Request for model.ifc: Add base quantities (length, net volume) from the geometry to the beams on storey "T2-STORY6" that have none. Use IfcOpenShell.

First a look at what the model holds.

```python
import ifcopenshell
import ifcopenshell.util.element
import ifcopenshell.util.unit

model = ifcopenshell.open("model.ifc")
print(model.schema)
for unit_type in ("LENGTHUNIT", "AREAUNIT", "VOLUMEUNIT"):
    print(unit_type, ifcopenshell.util.unit.calculate_unit_scale(model, unit_type))
storey = next(s for s in model.by_type("IfcBuildingStorey") if s.Name == "T2-STORY6")
beams = [e for e in ifcopenshell.util.element.get_decomposition(storey) if e.is_a("IfcBeam")]
for e in sorted(beams, key=lambda e: e.id()):
    print(e.id(), e.is_a(), e.Name, list(ifcopenshell.util.element.get_psets(e, qtos_only=True)), sep=" | ")
```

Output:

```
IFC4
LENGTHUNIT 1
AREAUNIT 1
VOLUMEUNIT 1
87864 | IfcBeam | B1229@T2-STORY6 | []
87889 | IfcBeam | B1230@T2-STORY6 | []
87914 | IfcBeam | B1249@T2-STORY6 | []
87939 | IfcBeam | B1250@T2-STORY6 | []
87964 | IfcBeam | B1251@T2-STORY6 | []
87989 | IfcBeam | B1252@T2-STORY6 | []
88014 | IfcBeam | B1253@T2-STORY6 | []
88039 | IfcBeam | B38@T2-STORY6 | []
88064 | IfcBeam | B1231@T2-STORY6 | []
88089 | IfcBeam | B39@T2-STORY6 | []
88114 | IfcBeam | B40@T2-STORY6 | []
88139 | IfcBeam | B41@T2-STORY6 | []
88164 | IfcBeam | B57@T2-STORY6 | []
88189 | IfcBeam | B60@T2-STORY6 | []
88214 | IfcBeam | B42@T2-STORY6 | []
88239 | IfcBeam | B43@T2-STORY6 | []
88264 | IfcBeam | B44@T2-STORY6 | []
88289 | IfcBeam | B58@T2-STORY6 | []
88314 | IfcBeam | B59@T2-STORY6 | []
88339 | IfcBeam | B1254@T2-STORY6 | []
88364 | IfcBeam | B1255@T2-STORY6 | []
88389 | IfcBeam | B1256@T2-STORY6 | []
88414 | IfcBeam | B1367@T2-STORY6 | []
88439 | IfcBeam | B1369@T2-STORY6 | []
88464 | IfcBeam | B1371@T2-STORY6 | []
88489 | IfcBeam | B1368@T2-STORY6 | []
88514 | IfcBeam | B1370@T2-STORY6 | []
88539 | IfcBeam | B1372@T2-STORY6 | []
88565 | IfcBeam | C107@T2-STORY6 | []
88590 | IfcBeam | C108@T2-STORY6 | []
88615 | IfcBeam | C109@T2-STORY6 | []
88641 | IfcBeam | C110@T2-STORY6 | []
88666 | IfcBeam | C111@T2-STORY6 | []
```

```python
import ifcopenshell
import ifcopenshell.api.pset
import ifcopenshell.geom
import ifcopenshell.util.element
import ifcopenshell.util.shape
import ifcopenshell.util.unit

model = ifcopenshell.open("model.ifc")
unit_scale = ifcopenshell.util.unit.calculate_unit_scale(model)
volume_scale = ifcopenshell.util.unit.calculate_unit_scale(model, "VOLUMEUNIT")
settings = ifcopenshell.geom.settings()

storey = next(s for s in model.by_type("IfcBuildingStorey") if s.Name == "T2-STORY6")
beams = [e for e in ifcopenshell.util.element.get_decomposition(storey) if e.is_a("IfcBeam")]

for e in sorted(beams, key=lambda e: e.id()):
    if ifcopenshell.util.element.get_psets(e, qtos_only=True, should_inherit=False):
        continue
    # Geometry comes back in metres, in the element's own axes.
    shape = ifcopenshell.geom.create_shape(settings, e)
    values = {
        "Length": ifcopenshell.util.shape.get_max_xyz(shape.geometry) / unit_scale,
        "NetVolume": ifcopenshell.util.shape.get_volume(shape.geometry) / volume_scale,
    }
    qto = ifcopenshell.api.pset.add_qto(model, product=e, name="Qto_BeamBaseQuantities")
    ifcopenshell.api.pset.edit_qto(model, qto=qto, properties=values)
    print(e.id(), {k: round(v, 3) for k, v in values.items()})

model.write("model_updated.ifc")
```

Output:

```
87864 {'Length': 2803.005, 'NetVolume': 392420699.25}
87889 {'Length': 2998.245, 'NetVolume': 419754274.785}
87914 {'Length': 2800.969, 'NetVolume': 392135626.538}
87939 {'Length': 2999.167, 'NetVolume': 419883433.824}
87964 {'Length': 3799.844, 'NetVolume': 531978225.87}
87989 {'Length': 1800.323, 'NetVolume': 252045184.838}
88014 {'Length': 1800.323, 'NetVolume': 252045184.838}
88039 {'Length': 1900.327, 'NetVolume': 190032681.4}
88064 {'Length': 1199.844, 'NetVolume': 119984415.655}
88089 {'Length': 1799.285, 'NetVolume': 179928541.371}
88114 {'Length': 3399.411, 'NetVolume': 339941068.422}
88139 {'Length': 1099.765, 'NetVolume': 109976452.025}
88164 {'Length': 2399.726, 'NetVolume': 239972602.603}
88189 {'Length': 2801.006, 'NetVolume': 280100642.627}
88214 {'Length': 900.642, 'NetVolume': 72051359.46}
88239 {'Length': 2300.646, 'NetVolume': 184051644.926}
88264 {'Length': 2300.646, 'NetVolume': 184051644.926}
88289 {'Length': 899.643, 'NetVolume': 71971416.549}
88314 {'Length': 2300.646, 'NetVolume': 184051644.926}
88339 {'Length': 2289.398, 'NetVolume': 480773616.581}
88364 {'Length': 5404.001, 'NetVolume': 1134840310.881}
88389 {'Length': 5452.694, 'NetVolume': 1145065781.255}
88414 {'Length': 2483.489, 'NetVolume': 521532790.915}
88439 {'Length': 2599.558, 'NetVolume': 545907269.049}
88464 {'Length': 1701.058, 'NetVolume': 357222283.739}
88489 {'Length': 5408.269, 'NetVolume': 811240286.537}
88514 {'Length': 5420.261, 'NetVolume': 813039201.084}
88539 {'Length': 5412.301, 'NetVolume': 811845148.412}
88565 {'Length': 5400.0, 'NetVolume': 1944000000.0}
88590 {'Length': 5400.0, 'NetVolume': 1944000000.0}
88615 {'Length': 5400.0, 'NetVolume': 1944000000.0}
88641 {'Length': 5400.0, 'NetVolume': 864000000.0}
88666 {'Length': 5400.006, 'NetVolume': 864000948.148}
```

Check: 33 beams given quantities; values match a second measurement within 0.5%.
